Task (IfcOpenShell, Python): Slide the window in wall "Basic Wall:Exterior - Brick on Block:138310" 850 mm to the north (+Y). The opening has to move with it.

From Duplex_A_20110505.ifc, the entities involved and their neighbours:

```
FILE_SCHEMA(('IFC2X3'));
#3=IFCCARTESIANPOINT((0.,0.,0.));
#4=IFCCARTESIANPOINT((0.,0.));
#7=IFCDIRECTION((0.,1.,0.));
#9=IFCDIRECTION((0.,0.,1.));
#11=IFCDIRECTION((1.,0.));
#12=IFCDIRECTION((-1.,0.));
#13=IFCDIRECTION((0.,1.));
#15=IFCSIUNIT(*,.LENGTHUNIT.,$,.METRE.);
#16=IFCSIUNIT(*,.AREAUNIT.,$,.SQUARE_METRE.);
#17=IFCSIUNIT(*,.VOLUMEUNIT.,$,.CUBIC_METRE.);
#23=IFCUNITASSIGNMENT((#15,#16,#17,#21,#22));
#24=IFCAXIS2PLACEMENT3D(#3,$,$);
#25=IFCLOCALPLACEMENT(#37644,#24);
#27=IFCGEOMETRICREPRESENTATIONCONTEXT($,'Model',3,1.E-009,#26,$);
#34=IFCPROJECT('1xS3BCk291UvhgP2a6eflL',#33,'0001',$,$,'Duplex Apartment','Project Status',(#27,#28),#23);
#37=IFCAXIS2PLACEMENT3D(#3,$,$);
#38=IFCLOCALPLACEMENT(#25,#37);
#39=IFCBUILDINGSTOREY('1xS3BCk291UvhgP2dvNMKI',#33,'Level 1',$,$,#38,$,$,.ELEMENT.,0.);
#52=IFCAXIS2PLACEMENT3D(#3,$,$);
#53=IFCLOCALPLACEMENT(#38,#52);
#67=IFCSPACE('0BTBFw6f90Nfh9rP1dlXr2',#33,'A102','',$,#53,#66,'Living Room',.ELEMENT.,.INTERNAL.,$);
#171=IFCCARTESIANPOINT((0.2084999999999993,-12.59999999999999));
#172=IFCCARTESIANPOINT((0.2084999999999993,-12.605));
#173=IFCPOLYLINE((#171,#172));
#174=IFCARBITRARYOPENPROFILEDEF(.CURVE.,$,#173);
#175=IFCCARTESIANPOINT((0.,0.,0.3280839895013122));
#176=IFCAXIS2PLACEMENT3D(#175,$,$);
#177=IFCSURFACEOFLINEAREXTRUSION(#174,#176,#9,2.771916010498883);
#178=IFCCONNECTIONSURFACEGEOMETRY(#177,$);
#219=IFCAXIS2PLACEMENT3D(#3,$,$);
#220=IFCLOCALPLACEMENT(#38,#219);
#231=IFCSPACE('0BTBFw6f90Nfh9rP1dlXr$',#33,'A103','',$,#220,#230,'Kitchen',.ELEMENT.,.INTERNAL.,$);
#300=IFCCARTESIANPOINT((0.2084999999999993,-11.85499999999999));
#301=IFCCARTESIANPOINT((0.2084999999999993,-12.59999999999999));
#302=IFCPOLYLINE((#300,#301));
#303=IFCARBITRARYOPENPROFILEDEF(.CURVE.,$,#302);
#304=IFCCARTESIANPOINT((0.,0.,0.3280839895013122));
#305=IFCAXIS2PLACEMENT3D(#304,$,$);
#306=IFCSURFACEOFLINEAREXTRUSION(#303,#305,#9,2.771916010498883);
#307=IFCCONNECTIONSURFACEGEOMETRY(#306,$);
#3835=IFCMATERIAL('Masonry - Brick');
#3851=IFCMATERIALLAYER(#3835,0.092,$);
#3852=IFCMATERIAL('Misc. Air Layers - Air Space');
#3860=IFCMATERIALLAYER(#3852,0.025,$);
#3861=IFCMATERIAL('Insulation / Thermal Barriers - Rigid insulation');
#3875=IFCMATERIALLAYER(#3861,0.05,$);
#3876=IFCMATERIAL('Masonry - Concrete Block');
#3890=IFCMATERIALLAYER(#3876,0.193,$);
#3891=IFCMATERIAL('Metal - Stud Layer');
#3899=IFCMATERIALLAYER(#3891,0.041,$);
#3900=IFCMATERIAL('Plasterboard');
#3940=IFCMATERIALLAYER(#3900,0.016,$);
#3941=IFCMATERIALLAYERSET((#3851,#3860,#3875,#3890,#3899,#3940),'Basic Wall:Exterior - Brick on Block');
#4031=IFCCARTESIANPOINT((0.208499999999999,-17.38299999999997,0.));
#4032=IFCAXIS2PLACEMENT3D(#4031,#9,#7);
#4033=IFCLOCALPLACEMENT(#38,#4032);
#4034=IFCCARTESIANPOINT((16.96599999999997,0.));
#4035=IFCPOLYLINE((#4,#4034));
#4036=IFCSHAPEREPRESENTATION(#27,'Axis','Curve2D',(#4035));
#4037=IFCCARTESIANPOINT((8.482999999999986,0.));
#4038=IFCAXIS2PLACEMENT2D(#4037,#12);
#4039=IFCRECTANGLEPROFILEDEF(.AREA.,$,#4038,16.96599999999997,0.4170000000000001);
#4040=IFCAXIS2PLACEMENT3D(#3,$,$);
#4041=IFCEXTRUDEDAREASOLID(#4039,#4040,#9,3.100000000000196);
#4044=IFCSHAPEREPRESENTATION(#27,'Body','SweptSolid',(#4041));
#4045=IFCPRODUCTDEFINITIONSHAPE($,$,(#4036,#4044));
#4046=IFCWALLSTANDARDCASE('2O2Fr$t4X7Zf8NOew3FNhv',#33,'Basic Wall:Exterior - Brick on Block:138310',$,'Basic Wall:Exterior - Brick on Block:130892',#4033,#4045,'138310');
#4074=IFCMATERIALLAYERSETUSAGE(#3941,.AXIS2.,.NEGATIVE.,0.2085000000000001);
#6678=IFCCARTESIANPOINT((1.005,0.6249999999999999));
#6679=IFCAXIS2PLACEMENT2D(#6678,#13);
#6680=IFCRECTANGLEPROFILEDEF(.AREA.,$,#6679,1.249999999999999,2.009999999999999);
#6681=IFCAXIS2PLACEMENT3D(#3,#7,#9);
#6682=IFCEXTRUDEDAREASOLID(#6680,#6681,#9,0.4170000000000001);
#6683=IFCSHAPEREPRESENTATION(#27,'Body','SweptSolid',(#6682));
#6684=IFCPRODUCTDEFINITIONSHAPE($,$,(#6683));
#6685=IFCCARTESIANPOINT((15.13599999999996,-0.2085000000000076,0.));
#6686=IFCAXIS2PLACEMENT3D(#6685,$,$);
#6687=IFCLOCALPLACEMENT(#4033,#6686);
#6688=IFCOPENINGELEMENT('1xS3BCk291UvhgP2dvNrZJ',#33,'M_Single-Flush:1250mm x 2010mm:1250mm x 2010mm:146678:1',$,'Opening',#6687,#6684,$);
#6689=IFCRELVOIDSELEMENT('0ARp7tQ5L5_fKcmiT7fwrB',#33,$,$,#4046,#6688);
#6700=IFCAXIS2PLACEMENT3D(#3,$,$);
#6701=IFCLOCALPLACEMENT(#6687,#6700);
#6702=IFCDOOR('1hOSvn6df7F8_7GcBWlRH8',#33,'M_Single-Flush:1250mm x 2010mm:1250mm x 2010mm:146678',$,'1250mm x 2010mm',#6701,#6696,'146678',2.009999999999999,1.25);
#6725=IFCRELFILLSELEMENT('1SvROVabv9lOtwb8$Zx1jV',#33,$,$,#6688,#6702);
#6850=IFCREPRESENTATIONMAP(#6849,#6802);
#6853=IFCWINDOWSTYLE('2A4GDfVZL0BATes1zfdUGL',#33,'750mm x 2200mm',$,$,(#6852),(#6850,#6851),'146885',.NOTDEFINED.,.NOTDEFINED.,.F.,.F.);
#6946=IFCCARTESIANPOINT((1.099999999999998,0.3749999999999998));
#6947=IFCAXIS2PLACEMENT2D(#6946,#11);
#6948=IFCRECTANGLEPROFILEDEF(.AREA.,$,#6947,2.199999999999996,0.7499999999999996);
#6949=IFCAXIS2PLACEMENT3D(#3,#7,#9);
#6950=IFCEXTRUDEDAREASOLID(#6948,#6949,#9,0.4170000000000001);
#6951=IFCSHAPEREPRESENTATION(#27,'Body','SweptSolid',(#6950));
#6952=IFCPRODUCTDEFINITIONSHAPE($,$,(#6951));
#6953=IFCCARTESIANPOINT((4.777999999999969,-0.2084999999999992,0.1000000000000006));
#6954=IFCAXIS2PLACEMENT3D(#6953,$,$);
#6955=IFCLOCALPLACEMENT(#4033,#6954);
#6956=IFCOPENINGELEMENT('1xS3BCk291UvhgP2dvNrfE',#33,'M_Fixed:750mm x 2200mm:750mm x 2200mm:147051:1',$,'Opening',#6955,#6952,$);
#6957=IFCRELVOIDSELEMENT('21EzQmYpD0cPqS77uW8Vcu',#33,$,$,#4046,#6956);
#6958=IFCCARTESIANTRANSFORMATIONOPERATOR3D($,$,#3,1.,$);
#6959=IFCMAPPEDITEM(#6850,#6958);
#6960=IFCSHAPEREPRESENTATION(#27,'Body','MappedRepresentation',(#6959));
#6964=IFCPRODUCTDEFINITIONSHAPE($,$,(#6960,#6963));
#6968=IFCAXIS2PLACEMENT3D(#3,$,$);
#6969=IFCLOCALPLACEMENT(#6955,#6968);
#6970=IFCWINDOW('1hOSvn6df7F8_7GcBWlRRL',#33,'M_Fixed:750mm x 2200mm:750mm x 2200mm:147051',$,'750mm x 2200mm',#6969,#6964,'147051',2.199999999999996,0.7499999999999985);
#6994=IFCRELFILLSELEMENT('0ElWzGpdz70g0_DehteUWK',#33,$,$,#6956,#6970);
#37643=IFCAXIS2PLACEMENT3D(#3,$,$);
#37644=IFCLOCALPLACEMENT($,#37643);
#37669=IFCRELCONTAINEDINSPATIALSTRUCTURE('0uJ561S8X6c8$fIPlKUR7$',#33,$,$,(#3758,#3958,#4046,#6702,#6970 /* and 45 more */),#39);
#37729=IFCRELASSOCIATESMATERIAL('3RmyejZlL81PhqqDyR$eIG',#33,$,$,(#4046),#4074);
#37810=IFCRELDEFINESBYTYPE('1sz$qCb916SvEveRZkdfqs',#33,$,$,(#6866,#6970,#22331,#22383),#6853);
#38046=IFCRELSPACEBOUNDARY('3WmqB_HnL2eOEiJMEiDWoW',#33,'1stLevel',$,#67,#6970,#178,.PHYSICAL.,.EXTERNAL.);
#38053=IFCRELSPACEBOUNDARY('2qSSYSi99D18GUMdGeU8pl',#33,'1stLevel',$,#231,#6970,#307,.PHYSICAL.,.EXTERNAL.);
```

```python
import numpy as np
import ifcopenshell
import ifcopenshell.api.geometry
import ifcopenshell.util.placement
import ifcopenshell.util.unit

model = ifcopenshell.open("Duplex_A_20110505.ifc")
unit_scale = ifcopenshell.util.unit.calculate_unit_scale(model)

window = model.by_guid("1hOSvn6df7F8_7GcBWlRRL")
opening = window.FillsVoids[0].RelatingOpeningElement
wall = opening.VoidsElements[0].RelatingBuildingElement

wall_matrix = ifcopenshell.util.placement.get_local_placement(wall.ObjectPlacement)
shift = wall_matrix[:3, 0] * 0.85 / unit_scale
before = ifcopenshell.util.placement.get_local_placement(window.ObjectPlacement)[:3, 3].copy()

# The window is placed relative to its opening, so it follows when the opening moves.
matrix = ifcopenshell.util.placement.get_local_placement(opening.ObjectPlacement)
matrix[:3, 3] += shift
ifcopenshell.api.geometry.edit_object_placement(
    model, product=opening, matrix=matrix, is_si=False, should_transform_children=True
)

# Space boundary surfaces are stored in each space's coordinates; move them too.
for rel in window.ProvidesBoundaries:
    if not rel.ConnectionGeometry:
        continue
    surface = rel.ConnectionGeometry.SurfaceOnRelatingElement
    space_matrix = ifcopenshell.util.placement.get_local_placement(rel.RelatingSpace.ObjectPlacement)
    point = np.array(surface.Position.Location.Coordinates) + space_matrix[:3, :3].T @ shift
    surface.Position = model.createIfcAxis2Placement3D(
        model.createIfcCartesianPoint(point.tolist()), surface.Position.Axis, surface.Position.RefDirection
    )

after = ifcopenshell.util.placement.get_local_placement(window.ObjectPlacement)[:3, 3]
print("window moved by", (after - before).round(3) + 0.0)

model.write("Duplex_A_20110505_v2.ifc")
```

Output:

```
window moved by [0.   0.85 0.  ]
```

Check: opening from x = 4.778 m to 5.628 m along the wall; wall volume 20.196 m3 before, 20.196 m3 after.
